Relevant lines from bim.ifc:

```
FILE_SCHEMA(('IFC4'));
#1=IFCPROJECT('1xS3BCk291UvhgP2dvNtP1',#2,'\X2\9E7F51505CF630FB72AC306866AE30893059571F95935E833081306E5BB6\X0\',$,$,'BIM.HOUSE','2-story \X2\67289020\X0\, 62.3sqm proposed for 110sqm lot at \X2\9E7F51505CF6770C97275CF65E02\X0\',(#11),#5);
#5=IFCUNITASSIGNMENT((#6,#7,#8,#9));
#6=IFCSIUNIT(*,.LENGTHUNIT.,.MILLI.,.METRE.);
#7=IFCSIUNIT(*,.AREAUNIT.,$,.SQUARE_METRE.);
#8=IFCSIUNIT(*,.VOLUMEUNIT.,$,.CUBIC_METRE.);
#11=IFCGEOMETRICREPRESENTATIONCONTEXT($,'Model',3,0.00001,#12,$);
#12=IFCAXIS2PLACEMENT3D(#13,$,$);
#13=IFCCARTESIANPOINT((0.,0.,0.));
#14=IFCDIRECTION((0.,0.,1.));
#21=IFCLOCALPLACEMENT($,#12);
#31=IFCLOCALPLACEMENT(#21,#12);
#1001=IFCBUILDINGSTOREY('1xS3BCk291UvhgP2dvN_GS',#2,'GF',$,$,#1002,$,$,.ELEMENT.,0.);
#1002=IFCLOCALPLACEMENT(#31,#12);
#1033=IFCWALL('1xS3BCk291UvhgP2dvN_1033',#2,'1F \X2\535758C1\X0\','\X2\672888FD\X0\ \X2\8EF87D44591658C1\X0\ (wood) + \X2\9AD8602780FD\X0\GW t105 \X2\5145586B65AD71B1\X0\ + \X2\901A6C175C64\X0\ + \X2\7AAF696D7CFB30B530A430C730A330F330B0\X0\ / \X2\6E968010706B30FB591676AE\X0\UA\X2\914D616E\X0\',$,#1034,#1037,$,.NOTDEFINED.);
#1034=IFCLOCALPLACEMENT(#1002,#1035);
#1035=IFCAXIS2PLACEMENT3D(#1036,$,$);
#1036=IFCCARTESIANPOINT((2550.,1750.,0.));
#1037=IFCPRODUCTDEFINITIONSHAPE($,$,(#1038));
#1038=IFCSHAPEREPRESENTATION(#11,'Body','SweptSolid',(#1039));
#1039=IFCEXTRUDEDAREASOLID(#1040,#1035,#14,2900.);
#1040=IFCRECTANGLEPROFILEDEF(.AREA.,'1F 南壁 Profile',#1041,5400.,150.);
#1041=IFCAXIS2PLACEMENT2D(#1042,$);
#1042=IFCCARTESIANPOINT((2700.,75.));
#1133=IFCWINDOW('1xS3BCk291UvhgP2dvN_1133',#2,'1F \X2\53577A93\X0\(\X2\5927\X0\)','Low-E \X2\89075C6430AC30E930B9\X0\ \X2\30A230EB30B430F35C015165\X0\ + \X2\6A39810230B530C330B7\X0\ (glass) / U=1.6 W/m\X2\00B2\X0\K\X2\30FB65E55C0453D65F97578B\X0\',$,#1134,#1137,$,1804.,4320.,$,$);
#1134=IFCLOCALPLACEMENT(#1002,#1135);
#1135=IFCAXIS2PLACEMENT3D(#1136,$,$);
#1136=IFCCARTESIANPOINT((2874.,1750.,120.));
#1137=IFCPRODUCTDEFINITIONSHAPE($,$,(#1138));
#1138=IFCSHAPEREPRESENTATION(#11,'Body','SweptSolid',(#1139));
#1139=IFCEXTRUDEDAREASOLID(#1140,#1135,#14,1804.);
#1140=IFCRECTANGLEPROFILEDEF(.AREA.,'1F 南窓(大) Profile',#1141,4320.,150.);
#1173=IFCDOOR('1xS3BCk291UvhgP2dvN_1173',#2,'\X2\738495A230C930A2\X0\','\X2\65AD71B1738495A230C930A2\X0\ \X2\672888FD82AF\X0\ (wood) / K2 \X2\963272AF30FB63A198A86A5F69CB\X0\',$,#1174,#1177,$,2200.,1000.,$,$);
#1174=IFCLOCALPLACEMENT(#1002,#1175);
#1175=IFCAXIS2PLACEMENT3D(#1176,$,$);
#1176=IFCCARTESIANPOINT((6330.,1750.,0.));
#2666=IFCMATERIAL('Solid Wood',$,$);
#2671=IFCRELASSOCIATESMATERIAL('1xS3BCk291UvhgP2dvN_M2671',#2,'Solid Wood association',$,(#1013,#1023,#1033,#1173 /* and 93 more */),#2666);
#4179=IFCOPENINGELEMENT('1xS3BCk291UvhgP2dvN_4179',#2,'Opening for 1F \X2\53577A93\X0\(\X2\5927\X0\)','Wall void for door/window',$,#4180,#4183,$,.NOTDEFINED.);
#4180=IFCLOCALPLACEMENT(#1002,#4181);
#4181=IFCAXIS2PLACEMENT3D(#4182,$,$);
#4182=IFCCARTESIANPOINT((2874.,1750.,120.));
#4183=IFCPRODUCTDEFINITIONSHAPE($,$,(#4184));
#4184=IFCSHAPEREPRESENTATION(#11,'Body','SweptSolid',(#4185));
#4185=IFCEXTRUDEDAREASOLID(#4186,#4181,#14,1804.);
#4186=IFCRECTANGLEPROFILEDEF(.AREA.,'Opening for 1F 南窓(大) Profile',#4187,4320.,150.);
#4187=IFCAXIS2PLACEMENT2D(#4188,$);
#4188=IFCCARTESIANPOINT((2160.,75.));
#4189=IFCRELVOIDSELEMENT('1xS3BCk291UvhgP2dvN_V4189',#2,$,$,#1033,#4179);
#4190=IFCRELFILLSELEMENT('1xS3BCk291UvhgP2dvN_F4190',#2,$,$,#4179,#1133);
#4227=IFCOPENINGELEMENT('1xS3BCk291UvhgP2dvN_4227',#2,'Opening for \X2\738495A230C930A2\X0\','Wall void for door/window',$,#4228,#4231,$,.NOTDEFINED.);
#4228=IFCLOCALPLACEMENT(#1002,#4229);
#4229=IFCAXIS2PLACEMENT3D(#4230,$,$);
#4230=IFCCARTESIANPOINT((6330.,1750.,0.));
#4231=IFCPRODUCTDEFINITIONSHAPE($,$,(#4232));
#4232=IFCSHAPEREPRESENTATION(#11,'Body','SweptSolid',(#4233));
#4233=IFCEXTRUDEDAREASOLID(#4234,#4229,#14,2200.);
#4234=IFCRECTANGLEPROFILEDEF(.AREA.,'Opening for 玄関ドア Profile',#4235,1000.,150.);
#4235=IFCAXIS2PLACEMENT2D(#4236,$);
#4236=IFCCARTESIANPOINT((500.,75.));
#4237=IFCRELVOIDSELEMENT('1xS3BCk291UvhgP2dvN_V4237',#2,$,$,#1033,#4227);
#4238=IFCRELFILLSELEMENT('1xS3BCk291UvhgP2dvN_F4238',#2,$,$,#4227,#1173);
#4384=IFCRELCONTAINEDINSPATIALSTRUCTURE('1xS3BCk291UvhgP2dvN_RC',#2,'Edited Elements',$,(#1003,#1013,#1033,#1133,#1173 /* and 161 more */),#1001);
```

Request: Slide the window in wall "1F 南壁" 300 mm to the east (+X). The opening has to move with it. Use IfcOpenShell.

```python
import ifcopenshell
import ifcopenshell.api.geometry
import ifcopenshell.util.placement

model = ifcopenshell.open("bim.ifc")

window = model.by_guid("1xS3BCk291UvhgP2dvN_1133")
opening = window.FillsVoids[0].RelatingOpeningElement
wall = opening.VoidsElements[0].RelatingBuildingElement

wall_matrix = ifcopenshell.util.placement.get_local_placement(wall.ObjectPlacement)
shift = wall_matrix[:3, 0] * 300.0
before = ifcopenshell.util.placement.get_local_placement(window.ObjectPlacement)[:3, 3].copy()

# The window is not placed relative to its opening, so move both.
for product in (opening, window):
    matrix = ifcopenshell.util.placement.get_local_placement(product.ObjectPlacement)
    matrix[:3, 3] += shift
    ifcopenshell.api.geometry.edit_object_placement(model, product=product, matrix=matrix, is_si=False)

after = ifcopenshell.util.placement.get_local_placement(window.ObjectPlacement)[:3, 3]
print("window moved by", (after - before).round(3) + 0.0)

model.write("bim_edited.ifc")
```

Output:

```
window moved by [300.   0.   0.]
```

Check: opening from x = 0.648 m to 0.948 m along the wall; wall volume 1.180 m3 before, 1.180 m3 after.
